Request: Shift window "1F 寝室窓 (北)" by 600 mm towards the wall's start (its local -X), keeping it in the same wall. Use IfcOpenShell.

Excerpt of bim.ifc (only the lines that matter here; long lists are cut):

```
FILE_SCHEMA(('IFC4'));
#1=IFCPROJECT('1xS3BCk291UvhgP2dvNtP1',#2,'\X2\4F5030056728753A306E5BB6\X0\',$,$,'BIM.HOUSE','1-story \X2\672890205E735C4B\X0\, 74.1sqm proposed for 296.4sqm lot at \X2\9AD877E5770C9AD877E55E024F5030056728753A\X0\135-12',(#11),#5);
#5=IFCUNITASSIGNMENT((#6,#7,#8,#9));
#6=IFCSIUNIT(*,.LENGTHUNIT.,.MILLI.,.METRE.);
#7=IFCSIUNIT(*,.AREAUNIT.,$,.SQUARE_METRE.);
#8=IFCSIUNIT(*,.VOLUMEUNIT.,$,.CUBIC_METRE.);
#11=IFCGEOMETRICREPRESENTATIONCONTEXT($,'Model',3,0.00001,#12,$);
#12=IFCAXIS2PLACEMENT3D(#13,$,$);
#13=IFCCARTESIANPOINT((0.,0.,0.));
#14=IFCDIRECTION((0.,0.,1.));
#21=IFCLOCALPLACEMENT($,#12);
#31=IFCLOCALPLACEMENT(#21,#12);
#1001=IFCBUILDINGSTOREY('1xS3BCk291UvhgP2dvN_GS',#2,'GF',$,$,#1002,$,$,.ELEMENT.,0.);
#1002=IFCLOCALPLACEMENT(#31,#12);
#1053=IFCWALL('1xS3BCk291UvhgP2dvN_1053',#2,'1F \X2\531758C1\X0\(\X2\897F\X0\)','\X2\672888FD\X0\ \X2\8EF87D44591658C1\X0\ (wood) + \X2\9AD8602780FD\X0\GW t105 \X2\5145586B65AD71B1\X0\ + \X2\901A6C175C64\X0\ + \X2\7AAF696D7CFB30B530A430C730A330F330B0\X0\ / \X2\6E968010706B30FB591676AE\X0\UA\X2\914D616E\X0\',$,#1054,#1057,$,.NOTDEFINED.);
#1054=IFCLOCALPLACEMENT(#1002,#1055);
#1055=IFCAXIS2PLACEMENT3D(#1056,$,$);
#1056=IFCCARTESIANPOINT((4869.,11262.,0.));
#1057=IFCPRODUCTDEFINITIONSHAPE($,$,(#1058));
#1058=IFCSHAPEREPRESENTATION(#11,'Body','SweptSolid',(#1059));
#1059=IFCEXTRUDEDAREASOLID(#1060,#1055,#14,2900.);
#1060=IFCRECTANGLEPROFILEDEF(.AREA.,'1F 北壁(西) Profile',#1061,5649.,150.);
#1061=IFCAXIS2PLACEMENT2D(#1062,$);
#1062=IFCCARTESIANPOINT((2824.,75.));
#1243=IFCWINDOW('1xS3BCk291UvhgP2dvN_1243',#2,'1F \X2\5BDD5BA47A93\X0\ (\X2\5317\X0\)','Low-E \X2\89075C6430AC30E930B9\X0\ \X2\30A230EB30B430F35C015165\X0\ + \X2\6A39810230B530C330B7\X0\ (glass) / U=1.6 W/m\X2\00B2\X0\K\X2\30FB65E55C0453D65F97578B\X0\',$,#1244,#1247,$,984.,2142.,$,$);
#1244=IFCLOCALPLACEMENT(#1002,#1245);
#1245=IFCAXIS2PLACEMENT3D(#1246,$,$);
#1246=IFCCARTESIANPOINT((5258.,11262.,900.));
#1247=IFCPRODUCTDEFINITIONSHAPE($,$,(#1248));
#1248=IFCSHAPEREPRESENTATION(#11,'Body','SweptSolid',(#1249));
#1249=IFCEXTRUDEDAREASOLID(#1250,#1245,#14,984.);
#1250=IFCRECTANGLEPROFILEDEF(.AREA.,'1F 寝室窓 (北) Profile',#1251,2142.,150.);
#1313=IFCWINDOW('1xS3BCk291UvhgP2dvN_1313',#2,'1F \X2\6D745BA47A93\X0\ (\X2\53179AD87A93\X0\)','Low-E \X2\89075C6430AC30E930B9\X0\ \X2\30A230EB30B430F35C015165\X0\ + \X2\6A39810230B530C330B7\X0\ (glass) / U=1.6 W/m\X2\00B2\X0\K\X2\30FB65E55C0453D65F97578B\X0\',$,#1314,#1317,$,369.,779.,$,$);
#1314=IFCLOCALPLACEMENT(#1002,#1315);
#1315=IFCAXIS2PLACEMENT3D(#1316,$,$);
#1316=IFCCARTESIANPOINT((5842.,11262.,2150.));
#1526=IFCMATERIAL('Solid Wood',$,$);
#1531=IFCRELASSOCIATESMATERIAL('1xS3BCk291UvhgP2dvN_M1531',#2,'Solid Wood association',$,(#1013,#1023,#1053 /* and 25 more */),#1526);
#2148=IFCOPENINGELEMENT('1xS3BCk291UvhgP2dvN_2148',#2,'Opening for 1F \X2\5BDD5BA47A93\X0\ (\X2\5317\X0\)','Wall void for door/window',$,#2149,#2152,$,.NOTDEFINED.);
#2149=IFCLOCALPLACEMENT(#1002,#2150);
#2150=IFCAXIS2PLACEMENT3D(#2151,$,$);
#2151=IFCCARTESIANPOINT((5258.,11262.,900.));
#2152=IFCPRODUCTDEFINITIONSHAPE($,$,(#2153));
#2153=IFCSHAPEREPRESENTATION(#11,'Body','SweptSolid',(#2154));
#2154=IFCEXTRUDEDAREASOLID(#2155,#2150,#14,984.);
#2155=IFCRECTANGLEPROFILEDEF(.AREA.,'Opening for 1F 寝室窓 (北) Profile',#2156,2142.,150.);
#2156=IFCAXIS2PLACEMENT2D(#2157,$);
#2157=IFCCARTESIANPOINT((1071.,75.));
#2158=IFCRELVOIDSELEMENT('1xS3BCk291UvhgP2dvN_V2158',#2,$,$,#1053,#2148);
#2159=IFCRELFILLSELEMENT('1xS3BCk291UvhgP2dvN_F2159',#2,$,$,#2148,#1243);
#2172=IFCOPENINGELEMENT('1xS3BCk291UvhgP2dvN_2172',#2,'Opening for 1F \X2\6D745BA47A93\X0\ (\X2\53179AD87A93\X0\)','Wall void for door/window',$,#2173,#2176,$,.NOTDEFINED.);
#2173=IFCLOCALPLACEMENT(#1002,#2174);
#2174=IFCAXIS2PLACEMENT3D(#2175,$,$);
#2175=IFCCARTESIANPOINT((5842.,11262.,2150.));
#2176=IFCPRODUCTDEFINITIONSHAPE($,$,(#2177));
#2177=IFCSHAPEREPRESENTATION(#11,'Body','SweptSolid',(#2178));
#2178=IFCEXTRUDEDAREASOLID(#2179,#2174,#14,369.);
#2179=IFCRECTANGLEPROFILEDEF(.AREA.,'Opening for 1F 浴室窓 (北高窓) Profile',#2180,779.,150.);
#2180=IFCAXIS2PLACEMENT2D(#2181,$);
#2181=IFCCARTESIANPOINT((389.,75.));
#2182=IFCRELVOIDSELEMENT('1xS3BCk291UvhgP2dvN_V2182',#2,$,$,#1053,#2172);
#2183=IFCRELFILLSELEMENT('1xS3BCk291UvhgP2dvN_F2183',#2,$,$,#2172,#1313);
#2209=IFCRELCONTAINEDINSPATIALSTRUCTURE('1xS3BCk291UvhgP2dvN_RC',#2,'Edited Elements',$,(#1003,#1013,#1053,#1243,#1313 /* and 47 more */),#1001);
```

```python
import ifcopenshell
import ifcopenshell.api.geometry
import ifcopenshell.util.placement
import ifcopenshell.util.unit

model = ifcopenshell.open("bim.ifc")
unit_scale = ifcopenshell.util.unit.calculate_unit_scale(model)

window = model.by_guid("1xS3BCk291UvhgP2dvN_1243")
opening = window.FillsVoids[0].RelatingOpeningElement
wall = opening.VoidsElements[0].RelatingBuildingElement

wall_matrix = ifcopenshell.util.placement.get_local_placement(wall.ObjectPlacement)
shift = wall_matrix[:3, 0] * -0.6 / unit_scale
before = ifcopenshell.util.placement.get_local_placement(window.ObjectPlacement)[:3, 3].copy()

# The window is not placed relative to its opening, so move both.
for product in (opening, window):
    matrix = ifcopenshell.util.placement.get_local_placement(product.ObjectPlacement)
    matrix[:3, 3] += shift
    ifcopenshell.api.geometry.edit_object_placement(model, product=product, matrix=matrix, is_si=False)

after = ifcopenshell.util.placement.get_local_placement(window.ObjectPlacement)[:3, 3]
print("window moved by", (after - before).round(3) + 0.0)

model.write("bim-out.ifc")
```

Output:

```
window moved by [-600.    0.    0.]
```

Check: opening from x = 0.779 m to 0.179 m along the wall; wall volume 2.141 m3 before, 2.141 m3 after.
